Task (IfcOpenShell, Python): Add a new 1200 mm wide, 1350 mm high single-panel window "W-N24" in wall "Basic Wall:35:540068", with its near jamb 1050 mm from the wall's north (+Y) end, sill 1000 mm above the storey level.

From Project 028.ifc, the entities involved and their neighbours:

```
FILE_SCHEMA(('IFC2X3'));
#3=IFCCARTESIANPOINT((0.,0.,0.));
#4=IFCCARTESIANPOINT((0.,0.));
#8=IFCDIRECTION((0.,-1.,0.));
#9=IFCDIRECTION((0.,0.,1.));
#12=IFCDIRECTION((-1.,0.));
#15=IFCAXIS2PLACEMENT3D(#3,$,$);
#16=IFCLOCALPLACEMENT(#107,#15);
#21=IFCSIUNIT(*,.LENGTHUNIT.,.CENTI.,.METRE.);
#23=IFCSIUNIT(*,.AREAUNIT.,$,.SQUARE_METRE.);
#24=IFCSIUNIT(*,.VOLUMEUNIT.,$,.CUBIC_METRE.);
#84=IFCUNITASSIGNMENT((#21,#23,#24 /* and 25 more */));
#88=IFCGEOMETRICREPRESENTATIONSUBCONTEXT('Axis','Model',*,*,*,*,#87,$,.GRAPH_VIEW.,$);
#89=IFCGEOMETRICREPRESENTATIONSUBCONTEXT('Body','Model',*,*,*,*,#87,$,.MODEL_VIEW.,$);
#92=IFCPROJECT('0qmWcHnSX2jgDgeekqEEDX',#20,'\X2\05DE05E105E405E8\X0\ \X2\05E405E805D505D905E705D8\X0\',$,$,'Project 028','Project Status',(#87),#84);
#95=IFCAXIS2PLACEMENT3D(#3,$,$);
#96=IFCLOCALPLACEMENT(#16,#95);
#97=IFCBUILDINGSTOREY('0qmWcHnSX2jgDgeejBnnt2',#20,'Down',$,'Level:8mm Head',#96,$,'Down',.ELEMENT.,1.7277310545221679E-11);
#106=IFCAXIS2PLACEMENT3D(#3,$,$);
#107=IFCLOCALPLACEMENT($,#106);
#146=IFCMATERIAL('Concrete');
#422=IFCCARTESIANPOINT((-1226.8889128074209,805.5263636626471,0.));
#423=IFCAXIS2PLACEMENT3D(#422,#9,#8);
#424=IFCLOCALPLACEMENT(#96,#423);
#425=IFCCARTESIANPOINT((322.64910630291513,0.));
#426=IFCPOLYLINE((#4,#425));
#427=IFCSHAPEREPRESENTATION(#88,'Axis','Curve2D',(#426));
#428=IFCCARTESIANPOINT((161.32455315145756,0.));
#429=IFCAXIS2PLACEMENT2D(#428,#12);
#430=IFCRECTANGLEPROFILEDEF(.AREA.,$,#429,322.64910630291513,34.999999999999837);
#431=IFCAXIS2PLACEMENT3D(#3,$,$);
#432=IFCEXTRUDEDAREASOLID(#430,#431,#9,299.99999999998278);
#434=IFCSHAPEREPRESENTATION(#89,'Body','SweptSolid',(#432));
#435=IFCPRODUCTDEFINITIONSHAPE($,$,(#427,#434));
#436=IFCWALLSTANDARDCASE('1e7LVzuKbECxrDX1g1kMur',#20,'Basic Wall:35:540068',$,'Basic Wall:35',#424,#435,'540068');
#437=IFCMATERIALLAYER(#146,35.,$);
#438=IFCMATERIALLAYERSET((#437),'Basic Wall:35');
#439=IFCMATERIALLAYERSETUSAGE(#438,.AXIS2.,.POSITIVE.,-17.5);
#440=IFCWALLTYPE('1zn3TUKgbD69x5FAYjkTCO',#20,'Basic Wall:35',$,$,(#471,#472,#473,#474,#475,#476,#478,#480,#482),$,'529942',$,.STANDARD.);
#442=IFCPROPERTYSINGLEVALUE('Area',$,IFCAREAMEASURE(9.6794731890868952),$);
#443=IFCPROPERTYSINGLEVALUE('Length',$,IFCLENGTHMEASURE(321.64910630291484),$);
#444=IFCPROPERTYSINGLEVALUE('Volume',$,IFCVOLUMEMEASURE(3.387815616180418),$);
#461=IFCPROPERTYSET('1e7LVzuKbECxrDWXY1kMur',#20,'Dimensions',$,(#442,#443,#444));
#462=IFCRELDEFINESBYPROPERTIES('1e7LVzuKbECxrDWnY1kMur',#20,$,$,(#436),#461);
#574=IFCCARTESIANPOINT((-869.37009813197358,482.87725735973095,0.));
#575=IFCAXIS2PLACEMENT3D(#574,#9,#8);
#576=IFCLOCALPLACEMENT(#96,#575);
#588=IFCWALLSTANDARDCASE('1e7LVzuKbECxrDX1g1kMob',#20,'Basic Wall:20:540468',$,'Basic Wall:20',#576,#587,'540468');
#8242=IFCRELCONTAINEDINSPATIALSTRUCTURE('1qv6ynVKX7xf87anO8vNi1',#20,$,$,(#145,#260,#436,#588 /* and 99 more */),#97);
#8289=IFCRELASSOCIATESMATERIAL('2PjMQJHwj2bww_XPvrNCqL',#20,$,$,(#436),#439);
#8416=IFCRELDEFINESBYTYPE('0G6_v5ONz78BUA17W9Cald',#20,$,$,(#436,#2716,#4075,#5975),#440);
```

```python
import numpy as np
import ifcopenshell
import ifcopenshell.api.feature
import ifcopenshell.api.geometry
import ifcopenshell.api.pset
import ifcopenshell.api.root
import ifcopenshell.api.spatial
import ifcopenshell.api.type
import ifcopenshell.geom
import ifcopenshell.util.element
import ifcopenshell.util.placement
import ifcopenshell.util.representation
import ifcopenshell.util.shape
import ifcopenshell.util.unit

model = ifcopenshell.open("Project 028.ifc")
unit_scale = ifcopenshell.util.unit.calculate_unit_scale(model)
area_scale = ifcopenshell.util.unit.calculate_unit_scale(model, "AREAUNIT")
volume_scale = ifcopenshell.util.unit.calculate_unit_scale(model, "VOLUMEUNIT")
settings = ifcopenshell.geom.settings()


def volume(element):
    """Net volume in cubic metres, openings subtracted."""
    shape = ifcopenshell.geom.create_shape(settings, element)
    return ifcopenshell.util.shape.get_volume(shape.geometry)


wall = model.by_guid("1e7LVzuKbECxrDX1g1kMur")
storey = ifcopenshell.util.element.get_container(wall, ifc_class="IfcBuildingStorey")
context = ifcopenshell.util.representation.get_context(model, "Model", "Body", "MODEL_VIEW")
before = volume(wall)

width, height, from_end, sill = 1.2, 1.35, 1.05, 1  # metres

# The wall runs along its own X axis, and the end named is its -X end.
wall_shape = ifcopenshell.geom.create_shape(settings, wall)
x, y, z = ifcopenshell.util.shape.get_vertices(wall_shape.geometry).T
start = x.min() + from_end
face, thickness = float(y.min()), float(y.max() - y.min())
wall_matrix = ifcopenshell.util.placement.get_local_placement(wall.ObjectPlacement)
level = ifcopenshell.util.placement.get_local_placement(storey.ObjectPlacement)[2, 3]


def in_wall(x, y):
    """Placement at x, y metres in the wall's axes, at sill height."""
    matrix = wall_matrix.copy()
    matrix[:, 3] = wall_matrix @ np.array([x / unit_scale, y / unit_scale, 0.0, 1.0])
    matrix[2, 3] = level + sill / unit_scale
    return matrix


# Opening: a box that overshoots both wall faces by 50 mm.
opening = ifcopenshell.api.root.create_entity(model, ifc_class="IfcOpeningElement")
box = ifcopenshell.api.geometry.add_wall_representation(
    model, context=context, length=width, height=height, thickness=thickness + 0.1
)
ifcopenshell.api.geometry.assign_representation(model, product=opening, representation=box)
ifcopenshell.api.geometry.edit_object_placement(model, product=opening, matrix=in_wall(start, face - 0.05), is_si=False)
ifcopenshell.api.feature.add_feature(model, feature=opening, element=wall)

window = ifcopenshell.api.root.create_entity(model, ifc_class="IfcWindow", name="W-N24")
window.OverallWidth, window.OverallHeight = width / unit_scale, height / unit_scale
body = ifcopenshell.api.geometry.add_window_representation(
    model,
    context=context,
    overall_width=window.OverallWidth,
    overall_height=window.OverallHeight,
    partition_type="SINGLE_PANEL",
)
ifcopenshell.api.geometry.assign_representation(model, product=window, representation=body)
ifcopenshell.api.spatial.assign_container(model, products=[window], relating_structure=storey)
fills = ifcopenshell.api.feature.add_filling(model, opening=opening, element=window)
fills.OwnerHistory = window.OwnerHistory  # required in IFC2X3

# IFC2X3 keeps the operation on the window style.
style = ifcopenshell.api.root.create_entity(model, ifc_class="IfcWindowStyle", name="W-N24")
style.OperationType, style.ConstructionType = "SINGLE_PANEL", "NOTDEFINED"
style.ParameterTakesPrecedence = style.Sizeable = False
ifcopenshell.api.type.assign_type(model, related_objects=[window], relating_type=style)

# Centre the window in the wall's thickness.
ifcopenshell.api.geometry.edit_object_placement(model, product=window, matrix=in_wall(start, face), is_si=False)
window_shape = ifcopenshell.geom.create_shape(settings, window)
depth = ifcopenshell.util.shape.get_vertices(window_shape.geometry)[:, 1]
offset = face + thickness / 2 - (depth.min() + depth.max()) / 2
ifcopenshell.api.geometry.edit_object_placement(model, product=window, matrix=in_wall(start, offset), is_si=False)

after = volume(wall)

# Update the wall's stored quantities.
pset = model.by_id(ifcopenshell.util.element.get_pset(wall, "Dimensions", should_inherit=False)["id"])
ifcopenshell.api.pset.edit_pset(model, pset=pset, properties={
    "Area": model.create_entity("IfcAreaMeasure", after / thickness / area_scale),
    "Volume": model.create_entity("IfcVolumeMeasure", after / volume_scale),
})

print(f"wall volume {before:.3f} -> {after:.3f} m3")

model.write("Project 028_rev.ifc")
```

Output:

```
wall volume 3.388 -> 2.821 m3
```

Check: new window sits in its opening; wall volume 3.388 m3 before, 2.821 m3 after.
